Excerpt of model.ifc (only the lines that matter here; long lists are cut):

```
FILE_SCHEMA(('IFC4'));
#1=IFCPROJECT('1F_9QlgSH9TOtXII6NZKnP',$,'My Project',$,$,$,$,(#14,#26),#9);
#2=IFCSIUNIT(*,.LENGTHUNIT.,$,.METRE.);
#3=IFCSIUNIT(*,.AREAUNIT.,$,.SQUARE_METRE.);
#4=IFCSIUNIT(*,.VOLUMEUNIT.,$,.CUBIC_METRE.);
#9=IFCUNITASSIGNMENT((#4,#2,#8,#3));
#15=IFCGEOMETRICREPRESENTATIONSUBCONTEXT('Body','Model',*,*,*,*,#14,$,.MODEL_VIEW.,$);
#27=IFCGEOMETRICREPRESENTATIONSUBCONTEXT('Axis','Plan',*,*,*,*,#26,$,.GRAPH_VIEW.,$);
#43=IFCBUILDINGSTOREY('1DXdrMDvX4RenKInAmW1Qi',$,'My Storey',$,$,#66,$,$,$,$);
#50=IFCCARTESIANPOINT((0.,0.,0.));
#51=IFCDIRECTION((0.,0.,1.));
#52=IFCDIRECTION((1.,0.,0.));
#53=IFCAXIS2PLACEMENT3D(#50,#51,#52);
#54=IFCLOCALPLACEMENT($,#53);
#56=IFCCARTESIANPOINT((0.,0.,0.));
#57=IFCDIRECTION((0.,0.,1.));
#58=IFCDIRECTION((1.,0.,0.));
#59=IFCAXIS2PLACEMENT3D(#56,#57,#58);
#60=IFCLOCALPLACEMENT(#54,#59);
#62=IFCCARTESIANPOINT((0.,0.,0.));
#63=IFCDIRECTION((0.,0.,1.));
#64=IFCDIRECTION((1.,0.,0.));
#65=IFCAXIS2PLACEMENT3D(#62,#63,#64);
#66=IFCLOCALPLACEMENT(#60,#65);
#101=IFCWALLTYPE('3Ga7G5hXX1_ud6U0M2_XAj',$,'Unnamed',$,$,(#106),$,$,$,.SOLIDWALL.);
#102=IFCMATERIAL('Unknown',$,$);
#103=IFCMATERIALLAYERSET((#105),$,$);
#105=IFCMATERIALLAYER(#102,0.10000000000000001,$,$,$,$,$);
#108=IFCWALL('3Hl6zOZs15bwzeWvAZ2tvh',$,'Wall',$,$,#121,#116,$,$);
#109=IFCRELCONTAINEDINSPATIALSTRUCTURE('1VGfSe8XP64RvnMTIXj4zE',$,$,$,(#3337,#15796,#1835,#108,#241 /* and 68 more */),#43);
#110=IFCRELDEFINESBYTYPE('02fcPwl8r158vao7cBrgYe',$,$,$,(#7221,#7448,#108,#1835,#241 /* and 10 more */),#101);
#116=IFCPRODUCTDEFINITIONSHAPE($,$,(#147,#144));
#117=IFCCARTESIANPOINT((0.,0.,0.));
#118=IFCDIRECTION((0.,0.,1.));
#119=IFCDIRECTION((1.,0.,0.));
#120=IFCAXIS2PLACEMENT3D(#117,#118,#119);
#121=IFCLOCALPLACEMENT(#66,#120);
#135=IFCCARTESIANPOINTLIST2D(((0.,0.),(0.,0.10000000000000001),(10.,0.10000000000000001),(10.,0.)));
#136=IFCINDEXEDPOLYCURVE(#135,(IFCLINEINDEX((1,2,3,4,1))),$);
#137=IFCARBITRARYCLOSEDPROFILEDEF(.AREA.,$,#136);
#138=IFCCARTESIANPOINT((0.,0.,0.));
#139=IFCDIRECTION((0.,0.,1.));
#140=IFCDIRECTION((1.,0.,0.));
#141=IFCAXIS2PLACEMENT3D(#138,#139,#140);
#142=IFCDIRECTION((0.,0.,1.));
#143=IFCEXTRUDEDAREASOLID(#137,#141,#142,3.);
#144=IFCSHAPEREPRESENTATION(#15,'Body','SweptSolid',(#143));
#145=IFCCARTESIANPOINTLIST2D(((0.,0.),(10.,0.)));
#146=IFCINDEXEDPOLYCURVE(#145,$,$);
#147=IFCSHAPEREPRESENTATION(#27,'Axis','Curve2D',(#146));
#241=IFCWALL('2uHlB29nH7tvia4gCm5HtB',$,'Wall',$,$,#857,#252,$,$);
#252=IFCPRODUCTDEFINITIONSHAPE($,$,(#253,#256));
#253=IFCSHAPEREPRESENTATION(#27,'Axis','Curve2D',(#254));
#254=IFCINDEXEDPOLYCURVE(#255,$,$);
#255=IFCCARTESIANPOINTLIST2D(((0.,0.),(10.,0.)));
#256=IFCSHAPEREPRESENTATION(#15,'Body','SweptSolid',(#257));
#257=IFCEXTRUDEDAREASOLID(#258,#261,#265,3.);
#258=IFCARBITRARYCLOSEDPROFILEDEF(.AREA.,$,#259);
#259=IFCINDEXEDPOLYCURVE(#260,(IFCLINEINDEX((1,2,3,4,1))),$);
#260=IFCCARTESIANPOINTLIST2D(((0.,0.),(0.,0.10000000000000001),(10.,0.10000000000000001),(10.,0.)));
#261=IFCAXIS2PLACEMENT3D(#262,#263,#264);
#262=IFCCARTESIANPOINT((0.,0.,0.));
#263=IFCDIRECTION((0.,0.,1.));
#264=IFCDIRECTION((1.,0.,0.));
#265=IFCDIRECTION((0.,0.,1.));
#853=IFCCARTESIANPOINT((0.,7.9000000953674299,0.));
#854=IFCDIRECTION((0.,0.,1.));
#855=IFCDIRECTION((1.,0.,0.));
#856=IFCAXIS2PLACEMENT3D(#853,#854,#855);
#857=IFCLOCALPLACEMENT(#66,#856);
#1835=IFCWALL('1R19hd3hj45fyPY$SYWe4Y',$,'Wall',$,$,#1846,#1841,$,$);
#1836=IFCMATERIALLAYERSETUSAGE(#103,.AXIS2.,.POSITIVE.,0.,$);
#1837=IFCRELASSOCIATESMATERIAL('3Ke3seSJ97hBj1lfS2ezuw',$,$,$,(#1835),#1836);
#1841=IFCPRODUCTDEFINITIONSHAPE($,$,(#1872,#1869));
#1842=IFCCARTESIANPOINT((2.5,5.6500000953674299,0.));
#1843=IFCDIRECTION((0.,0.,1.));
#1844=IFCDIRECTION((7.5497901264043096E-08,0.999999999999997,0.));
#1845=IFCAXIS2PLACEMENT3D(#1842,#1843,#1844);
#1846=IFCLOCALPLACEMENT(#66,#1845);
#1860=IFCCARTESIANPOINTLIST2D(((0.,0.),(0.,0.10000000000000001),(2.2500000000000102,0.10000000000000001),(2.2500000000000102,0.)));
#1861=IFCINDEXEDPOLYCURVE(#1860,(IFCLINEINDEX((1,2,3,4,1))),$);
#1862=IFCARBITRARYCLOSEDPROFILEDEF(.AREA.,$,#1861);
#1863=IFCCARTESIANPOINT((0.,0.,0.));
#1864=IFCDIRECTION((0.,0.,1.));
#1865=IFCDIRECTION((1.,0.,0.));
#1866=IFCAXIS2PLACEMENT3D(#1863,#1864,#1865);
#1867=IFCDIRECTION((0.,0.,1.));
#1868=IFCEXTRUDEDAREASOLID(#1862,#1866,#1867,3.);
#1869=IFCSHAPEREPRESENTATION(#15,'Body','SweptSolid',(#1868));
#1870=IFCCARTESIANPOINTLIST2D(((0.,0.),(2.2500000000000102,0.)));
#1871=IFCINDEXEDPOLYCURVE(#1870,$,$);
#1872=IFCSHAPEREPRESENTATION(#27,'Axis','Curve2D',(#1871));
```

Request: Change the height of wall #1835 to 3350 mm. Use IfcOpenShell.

```python
import ifcopenshell
import ifcopenshell.geom
import ifcopenshell.util.representation
import ifcopenshell.util.shape

model = ifcopenshell.open("model.ifc")
settings = ifcopenshell.geom.settings()


def volume(element):
    """Net volume in cubic metres, openings subtracted."""
    shape = ifcopenshell.geom.create_shape(settings, element)
    return ifcopenshell.util.shape.get_volume(shape.geometry)


wall = model.by_id(1835)
before = volume(wall)

body = ifcopenshell.util.representation.get_representation(wall, "Model", "Body")
solid = body.Items[0]
old_height = solid.Depth
solid.Depth = 3.35
after = volume(wall)

print(f"height {old_height:g} -> {solid.Depth:g}, volume {before:.3f} -> {after:.3f} m3")

model.write("model_rev.ifc")
```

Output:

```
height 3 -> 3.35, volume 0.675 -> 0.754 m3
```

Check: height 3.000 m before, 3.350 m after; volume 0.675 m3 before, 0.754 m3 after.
